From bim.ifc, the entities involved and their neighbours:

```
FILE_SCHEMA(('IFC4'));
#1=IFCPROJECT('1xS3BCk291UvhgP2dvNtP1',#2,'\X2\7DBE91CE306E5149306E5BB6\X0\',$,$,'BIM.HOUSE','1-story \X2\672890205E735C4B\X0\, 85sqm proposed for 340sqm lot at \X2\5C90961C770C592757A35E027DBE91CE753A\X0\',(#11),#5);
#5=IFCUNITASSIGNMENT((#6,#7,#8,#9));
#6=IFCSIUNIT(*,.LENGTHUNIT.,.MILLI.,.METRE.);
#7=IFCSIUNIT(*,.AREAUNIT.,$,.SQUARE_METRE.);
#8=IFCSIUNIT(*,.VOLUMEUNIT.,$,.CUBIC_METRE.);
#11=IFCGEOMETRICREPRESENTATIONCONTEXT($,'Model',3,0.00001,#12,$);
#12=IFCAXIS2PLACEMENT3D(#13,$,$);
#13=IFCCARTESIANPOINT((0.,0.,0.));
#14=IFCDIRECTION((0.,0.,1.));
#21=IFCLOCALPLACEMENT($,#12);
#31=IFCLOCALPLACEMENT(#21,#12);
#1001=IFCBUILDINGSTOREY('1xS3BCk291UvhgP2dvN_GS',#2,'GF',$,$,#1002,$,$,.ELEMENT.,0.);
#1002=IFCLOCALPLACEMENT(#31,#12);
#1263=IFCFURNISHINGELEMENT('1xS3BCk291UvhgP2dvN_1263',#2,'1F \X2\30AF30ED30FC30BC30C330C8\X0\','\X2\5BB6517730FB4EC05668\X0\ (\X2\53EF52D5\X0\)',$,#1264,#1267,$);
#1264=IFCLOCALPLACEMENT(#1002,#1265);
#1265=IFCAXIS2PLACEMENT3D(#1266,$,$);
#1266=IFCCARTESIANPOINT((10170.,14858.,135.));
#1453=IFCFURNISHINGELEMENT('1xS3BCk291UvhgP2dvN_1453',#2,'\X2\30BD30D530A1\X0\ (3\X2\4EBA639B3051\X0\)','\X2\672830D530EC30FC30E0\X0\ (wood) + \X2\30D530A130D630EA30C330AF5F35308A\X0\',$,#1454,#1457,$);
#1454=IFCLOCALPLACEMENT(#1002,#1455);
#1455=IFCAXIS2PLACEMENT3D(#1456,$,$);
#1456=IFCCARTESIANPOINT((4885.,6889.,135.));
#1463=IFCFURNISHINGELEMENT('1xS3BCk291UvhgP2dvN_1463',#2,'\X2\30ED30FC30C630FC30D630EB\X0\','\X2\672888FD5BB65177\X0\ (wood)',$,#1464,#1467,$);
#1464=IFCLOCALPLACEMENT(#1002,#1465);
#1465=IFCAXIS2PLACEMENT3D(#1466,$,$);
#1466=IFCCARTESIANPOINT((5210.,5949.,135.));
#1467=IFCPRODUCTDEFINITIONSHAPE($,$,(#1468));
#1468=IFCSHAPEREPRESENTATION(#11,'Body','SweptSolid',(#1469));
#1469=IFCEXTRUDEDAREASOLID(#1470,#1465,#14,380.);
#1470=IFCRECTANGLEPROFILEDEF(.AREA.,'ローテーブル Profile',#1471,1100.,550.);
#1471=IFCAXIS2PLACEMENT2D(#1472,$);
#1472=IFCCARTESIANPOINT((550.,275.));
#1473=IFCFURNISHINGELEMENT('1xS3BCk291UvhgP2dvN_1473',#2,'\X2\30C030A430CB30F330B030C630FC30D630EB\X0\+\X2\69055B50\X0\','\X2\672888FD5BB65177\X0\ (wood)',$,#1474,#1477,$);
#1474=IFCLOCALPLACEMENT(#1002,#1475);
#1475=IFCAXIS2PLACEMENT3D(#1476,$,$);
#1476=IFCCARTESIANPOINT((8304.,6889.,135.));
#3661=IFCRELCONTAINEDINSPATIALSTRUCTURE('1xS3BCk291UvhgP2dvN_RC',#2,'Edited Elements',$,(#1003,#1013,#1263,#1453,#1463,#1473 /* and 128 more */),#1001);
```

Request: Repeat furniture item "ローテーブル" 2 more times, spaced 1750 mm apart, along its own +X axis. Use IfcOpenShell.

```python
import ifcopenshell
import ifcopenshell.api.geometry
import ifcopenshell.api.root
import ifcopenshell.util.element
import ifcopenshell.util.placement
import ifcopenshell.util.unit

model = ifcopenshell.open("bim.ifc")
unit_scale = ifcopenshell.util.unit.calculate_unit_scale(model)


def reuse_history(source, copy):
    """copy_class also copies each property set's owner history, people and application; keep the originals."""
    for rel in copy.IsDefinedBy:
        if rel.is_a("IfcRelDefinesByProperties") and (history := rel.RelatingPropertyDefinition.OwnerHistory):
            rel.RelatingPropertyDefinition.OwnerHistory = source.OwnerHistory
            ifcopenshell.util.element.remove_deep2(model, history)


source = model.by_guid("1xS3BCk291UvhgP2dvN_1463")
base = ifcopenshell.util.placement.get_local_placement(source.ObjectPlacement)
step = base[:3, 0] * 1.75 / unit_scale

for i in range(1, 3):
    copy = ifcopenshell.api.root.copy_class(model, product=source)
    copy.Representation = ifcopenshell.util.element.copy_deep(
        model, source.Representation, exclude=["IfcGeometricRepresentationContext", "IfcRepresentationMap"]
    )
    reuse_history(source, copy)
    matrix = base.copy()
    matrix[:3, 3] += i * step
    print("added at", matrix[:3, 3].round(3) + 0.0)
    ifcopenshell.api.geometry.edit_object_placement(model, product=copy, matrix=matrix, is_si=False)

model.write("bim_rev.ifc")
```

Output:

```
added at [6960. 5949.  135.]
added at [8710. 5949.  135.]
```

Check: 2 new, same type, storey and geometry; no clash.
